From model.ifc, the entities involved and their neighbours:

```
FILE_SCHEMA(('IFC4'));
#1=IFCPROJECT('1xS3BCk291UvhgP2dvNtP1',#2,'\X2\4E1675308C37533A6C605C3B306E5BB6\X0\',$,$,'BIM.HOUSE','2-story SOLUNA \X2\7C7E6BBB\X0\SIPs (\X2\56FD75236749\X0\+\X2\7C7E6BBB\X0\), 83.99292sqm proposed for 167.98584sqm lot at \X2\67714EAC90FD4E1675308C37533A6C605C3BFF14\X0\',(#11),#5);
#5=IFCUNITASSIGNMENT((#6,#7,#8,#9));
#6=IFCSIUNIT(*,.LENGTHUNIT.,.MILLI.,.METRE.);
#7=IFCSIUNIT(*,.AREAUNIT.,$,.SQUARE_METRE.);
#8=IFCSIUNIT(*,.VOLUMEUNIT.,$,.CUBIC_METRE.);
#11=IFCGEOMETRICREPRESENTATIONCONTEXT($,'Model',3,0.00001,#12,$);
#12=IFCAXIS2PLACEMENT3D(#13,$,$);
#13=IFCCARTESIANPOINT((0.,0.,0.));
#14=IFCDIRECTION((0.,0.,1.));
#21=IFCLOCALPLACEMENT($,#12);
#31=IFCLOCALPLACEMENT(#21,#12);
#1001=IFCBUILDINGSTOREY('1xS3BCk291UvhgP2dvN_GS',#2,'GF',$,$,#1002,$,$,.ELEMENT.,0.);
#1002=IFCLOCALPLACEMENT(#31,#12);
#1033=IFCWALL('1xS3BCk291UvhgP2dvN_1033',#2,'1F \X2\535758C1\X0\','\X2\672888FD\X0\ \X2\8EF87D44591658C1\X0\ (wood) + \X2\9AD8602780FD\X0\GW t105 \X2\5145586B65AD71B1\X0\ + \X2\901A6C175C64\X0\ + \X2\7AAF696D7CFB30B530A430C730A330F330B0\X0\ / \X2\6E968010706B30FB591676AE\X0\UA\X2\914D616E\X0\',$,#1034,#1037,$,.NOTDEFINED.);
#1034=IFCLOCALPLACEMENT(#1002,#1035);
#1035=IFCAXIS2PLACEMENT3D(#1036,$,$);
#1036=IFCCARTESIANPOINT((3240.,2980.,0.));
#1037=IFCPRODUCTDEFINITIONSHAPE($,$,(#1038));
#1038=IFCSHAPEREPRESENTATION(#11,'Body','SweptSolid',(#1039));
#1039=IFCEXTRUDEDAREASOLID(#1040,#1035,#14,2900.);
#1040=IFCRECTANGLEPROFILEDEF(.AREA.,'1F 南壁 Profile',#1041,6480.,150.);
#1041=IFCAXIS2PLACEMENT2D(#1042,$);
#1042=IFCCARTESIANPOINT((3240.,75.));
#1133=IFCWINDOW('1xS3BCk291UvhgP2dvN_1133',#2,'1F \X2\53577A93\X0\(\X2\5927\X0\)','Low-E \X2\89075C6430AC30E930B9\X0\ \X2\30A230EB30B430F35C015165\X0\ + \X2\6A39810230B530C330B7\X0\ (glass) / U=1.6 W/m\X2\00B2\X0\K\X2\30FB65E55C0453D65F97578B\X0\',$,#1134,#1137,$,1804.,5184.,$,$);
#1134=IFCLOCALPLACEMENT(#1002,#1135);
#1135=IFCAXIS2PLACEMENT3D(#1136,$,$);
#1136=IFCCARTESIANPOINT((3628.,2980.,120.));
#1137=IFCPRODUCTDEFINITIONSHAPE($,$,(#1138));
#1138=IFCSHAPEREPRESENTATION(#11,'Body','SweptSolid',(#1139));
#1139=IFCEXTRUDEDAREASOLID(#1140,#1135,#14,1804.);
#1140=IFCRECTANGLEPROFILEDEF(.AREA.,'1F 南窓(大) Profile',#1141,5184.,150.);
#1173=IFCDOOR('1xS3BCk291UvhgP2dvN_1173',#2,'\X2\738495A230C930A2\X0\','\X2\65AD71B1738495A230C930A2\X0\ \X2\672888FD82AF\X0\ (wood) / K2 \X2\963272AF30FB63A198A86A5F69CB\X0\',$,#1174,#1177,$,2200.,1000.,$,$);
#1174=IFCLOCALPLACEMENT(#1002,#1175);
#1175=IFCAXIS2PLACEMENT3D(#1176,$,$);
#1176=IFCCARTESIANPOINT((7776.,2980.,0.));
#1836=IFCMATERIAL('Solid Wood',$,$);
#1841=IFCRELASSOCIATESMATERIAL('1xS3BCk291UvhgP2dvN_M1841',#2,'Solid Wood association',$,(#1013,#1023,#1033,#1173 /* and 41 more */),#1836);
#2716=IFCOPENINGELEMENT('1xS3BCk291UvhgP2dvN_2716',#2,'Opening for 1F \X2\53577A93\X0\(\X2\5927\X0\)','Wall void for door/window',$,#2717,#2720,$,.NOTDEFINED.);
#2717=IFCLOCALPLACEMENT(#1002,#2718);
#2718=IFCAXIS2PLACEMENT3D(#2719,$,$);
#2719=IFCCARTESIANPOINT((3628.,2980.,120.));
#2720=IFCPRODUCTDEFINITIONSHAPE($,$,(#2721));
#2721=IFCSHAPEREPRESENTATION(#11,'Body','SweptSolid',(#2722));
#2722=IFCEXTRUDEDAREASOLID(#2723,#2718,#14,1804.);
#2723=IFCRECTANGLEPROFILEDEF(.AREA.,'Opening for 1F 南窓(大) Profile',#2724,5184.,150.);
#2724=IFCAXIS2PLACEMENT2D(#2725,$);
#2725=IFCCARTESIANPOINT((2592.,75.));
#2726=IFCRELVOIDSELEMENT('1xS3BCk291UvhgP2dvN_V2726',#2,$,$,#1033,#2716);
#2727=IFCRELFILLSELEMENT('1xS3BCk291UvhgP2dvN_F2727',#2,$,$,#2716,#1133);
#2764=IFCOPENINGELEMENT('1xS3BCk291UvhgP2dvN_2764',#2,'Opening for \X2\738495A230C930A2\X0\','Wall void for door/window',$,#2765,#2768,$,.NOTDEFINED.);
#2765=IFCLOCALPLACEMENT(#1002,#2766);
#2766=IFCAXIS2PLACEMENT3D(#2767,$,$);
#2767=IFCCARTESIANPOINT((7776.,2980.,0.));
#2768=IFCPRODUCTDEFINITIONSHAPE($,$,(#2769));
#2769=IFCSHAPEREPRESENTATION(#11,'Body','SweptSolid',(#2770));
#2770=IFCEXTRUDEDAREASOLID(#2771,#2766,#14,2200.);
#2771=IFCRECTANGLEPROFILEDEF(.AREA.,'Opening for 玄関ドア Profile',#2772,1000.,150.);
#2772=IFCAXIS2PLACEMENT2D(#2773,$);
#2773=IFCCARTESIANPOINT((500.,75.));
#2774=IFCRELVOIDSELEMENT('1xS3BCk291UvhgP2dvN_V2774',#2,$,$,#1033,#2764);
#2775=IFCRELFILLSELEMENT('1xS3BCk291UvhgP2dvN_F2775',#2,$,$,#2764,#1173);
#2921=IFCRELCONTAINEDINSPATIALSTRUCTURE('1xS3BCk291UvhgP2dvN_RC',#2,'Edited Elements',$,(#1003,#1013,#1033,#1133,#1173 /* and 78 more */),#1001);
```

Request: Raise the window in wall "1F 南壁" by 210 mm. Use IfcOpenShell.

```python
import numpy as np
import ifcopenshell
import ifcopenshell.api.geometry
import ifcopenshell.util.placement
import ifcopenshell.util.unit

model = ifcopenshell.open("model.ifc")
unit_scale = ifcopenshell.util.unit.calculate_unit_scale(model)

window = model.by_id(1133)
opening = window.FillsVoids[0].RelatingOpeningElement
dz = 0.21 / unit_scale

shift = np.array([0.0, 0.0, dz])
# The window is not placed relative to its opening, so move both.
for product in (opening, window):
    matrix = ifcopenshell.util.placement.get_local_placement(product.ObjectPlacement)
    matrix[:3, 3] += shift
    ifcopenshell.api.geometry.edit_object_placement(model, product=product, matrix=matrix, is_si=False)

print(f"moved by {dz * unit_scale:+.3f} m")

model.write("model-out.ifc")
```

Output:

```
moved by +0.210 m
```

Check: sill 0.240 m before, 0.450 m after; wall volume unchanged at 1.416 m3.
